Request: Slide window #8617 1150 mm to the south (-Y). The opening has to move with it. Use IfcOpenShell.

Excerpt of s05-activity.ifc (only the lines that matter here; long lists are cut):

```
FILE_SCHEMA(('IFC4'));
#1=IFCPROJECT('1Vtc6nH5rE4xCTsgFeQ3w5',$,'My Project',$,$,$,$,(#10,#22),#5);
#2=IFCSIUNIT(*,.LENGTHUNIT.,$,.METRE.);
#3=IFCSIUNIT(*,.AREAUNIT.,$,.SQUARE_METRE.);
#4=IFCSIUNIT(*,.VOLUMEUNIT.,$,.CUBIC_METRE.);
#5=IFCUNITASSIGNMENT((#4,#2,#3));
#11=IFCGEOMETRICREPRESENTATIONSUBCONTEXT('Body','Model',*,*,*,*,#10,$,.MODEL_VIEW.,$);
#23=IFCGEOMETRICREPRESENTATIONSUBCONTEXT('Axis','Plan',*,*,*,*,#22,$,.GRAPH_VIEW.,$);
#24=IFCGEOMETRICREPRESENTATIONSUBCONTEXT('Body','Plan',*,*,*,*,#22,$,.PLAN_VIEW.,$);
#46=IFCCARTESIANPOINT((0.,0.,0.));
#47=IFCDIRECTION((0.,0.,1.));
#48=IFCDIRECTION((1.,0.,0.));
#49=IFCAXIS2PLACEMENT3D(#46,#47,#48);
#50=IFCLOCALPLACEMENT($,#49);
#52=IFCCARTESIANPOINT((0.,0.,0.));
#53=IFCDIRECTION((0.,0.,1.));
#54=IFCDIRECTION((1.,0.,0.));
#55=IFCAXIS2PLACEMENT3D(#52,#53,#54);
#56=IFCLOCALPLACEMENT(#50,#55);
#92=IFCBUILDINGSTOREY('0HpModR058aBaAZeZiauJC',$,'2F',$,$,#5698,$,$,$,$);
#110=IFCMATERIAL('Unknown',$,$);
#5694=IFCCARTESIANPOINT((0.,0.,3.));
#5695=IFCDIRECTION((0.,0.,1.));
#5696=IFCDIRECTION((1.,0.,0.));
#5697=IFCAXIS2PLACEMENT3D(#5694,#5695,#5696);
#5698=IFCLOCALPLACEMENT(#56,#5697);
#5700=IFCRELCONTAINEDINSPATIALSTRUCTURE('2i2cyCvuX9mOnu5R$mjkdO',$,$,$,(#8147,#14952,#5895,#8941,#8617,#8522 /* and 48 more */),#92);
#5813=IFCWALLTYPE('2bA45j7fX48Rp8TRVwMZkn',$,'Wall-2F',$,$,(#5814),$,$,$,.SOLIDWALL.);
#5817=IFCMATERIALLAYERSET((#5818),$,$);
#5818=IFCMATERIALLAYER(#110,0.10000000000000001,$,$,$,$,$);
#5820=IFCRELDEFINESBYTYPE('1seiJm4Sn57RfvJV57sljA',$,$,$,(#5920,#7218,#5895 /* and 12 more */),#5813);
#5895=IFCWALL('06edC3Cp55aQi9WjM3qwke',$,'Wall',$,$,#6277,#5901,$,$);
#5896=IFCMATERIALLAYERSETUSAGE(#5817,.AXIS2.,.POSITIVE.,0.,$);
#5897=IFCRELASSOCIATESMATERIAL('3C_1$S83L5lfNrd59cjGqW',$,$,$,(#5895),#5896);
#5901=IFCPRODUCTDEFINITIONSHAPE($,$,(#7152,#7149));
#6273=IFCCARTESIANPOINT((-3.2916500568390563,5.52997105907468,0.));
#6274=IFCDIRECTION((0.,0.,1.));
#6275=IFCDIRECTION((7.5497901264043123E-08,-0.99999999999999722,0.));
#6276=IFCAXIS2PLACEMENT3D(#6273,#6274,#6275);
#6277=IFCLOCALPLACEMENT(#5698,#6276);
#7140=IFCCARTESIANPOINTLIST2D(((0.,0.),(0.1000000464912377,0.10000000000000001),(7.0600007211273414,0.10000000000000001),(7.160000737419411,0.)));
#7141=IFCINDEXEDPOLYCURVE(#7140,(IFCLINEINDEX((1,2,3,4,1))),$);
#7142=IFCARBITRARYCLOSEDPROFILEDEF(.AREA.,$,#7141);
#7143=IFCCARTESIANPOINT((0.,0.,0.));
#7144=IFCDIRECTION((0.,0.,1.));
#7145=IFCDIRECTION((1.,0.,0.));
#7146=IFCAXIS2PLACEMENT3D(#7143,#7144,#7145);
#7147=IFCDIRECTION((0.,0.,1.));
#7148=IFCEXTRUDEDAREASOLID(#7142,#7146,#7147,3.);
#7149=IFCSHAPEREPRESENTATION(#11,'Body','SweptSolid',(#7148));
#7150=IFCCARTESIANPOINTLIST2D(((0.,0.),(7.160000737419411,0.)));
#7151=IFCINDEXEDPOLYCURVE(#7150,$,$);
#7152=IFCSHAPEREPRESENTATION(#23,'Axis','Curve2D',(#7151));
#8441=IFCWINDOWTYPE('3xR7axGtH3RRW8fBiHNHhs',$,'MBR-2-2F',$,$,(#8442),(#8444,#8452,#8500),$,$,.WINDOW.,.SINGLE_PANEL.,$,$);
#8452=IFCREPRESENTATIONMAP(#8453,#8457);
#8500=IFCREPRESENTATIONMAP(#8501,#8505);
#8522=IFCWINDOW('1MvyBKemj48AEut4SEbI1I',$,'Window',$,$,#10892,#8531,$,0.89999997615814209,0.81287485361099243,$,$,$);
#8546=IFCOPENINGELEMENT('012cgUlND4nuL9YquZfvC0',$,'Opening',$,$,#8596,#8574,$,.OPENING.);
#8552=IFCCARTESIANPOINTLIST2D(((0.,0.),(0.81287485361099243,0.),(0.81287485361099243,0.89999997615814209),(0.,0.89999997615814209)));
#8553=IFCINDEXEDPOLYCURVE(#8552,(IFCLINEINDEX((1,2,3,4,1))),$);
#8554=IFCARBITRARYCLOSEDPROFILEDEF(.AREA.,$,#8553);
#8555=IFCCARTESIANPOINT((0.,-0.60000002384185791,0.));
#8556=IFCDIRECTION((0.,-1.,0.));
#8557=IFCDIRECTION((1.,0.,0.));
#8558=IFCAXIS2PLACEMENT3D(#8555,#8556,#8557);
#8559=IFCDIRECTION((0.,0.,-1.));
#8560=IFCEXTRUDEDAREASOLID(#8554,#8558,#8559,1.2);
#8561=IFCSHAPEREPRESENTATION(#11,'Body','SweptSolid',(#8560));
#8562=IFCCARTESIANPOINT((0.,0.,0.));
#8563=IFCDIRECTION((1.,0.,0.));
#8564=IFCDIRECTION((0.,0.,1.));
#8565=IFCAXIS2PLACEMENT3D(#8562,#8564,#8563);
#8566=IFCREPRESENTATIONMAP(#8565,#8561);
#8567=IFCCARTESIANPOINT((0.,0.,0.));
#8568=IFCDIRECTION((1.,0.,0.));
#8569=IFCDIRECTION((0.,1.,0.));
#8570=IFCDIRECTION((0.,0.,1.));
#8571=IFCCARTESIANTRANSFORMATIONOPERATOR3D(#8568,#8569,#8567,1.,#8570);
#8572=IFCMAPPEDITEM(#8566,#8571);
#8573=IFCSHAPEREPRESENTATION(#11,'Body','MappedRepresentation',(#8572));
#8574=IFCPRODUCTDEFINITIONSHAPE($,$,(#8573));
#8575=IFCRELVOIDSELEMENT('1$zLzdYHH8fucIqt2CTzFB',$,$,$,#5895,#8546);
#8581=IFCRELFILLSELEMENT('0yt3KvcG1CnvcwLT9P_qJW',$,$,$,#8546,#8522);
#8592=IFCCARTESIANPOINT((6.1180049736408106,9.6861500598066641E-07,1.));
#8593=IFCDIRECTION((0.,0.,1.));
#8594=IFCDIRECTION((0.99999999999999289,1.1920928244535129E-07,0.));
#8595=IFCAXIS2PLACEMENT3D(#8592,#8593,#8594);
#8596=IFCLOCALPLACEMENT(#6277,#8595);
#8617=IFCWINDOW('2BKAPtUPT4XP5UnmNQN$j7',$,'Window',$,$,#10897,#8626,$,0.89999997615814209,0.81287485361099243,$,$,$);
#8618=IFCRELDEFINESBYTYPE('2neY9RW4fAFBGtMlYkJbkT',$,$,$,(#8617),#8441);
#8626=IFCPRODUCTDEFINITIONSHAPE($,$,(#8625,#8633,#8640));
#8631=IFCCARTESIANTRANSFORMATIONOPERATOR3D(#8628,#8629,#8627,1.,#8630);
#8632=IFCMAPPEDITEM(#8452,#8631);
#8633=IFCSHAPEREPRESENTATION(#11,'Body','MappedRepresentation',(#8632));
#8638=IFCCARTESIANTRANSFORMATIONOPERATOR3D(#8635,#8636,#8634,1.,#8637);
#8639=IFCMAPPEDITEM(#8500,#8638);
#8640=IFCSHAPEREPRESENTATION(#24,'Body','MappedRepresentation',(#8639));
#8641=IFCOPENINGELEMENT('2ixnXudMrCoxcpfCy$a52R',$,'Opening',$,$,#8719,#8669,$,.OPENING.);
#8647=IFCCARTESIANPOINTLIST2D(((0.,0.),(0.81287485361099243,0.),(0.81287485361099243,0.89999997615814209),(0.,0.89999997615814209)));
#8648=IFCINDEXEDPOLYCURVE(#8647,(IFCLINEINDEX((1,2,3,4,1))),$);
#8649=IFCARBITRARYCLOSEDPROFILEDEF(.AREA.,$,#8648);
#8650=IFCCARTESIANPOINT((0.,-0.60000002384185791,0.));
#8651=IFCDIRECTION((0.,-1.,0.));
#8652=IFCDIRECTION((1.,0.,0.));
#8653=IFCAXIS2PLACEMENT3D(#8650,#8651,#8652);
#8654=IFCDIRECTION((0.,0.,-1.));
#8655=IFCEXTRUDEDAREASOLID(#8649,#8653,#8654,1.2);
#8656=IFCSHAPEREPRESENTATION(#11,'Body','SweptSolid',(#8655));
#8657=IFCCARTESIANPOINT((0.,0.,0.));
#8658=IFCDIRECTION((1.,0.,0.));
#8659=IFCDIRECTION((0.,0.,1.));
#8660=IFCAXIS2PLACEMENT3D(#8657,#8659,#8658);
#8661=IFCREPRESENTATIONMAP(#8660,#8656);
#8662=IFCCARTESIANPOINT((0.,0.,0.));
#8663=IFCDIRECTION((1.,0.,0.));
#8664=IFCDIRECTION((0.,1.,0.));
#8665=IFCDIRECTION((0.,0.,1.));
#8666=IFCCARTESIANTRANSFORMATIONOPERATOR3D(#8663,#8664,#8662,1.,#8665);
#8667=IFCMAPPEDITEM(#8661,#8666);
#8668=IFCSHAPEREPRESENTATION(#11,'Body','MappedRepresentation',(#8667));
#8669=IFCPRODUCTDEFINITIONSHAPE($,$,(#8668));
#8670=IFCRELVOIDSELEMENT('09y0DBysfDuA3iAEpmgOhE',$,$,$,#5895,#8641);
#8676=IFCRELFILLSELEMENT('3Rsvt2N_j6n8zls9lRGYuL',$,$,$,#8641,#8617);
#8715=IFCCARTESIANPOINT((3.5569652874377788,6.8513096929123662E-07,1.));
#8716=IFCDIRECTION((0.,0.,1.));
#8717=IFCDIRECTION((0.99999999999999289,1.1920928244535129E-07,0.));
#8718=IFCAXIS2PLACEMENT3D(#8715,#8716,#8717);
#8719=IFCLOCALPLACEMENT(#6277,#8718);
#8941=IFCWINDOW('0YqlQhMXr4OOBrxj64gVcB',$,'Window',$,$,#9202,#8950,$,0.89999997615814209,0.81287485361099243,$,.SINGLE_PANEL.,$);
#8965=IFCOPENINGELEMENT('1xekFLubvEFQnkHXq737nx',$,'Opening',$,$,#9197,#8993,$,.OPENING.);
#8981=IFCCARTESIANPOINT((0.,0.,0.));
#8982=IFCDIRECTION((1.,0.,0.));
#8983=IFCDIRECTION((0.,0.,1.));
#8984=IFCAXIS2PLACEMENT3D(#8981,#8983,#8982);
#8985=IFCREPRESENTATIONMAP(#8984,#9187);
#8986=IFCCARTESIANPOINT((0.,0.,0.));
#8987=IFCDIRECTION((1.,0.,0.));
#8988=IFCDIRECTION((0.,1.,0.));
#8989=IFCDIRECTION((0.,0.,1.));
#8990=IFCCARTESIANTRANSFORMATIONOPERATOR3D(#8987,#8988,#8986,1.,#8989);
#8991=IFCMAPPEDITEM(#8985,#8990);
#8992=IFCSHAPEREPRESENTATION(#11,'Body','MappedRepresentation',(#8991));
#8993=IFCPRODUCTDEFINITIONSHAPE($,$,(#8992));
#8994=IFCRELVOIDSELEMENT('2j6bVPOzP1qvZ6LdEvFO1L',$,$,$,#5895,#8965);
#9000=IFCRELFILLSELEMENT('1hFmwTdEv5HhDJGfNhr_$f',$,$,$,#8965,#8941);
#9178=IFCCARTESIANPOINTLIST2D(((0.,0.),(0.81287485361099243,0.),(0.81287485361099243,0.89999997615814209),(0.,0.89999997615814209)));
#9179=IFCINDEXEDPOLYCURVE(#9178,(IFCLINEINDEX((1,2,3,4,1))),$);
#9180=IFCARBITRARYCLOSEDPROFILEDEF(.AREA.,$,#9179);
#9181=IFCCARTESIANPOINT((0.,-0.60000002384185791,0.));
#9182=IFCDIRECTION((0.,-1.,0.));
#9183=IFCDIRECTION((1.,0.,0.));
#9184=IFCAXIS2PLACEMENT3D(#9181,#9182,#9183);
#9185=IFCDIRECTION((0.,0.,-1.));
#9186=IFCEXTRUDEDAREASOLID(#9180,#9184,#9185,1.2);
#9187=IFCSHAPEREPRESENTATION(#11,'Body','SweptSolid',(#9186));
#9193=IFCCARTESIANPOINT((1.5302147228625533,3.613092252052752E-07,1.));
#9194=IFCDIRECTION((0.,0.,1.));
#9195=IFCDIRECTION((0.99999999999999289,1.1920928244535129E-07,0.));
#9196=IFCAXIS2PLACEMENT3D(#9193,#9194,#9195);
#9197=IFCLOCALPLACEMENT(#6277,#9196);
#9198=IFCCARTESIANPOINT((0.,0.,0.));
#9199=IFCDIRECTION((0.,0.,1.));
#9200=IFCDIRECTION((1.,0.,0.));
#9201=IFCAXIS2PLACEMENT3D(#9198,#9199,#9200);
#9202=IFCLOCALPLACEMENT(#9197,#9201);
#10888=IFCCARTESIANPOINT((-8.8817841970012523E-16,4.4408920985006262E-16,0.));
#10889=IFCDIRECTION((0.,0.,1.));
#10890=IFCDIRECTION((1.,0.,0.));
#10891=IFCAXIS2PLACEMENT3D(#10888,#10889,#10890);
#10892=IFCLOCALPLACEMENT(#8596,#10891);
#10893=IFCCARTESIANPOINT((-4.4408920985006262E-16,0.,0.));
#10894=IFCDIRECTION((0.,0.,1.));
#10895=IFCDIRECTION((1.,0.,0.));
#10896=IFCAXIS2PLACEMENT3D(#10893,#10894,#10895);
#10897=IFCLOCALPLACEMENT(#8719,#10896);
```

```python
import ifcopenshell
import ifcopenshell.api.geometry
import ifcopenshell.util.placement
import ifcopenshell.util.unit

model = ifcopenshell.open("s05-activity.ifc")
unit_scale = ifcopenshell.util.unit.calculate_unit_scale(model)

window = model.by_guid("2BKAPtUPT4XP5UnmNQN$j7")
opening = window.FillsVoids[0].RelatingOpeningElement
wall = opening.VoidsElements[0].RelatingBuildingElement

wall_matrix = ifcopenshell.util.placement.get_local_placement(wall.ObjectPlacement)
shift = wall_matrix[:3, 0] * 1.15 / unit_scale
before = ifcopenshell.util.placement.get_local_placement(window.ObjectPlacement)[:3, 3].copy()

# The window is placed relative to its opening, so it follows when the opening moves.
matrix = ifcopenshell.util.placement.get_local_placement(opening.ObjectPlacement)
matrix[:3, 3] += shift
ifcopenshell.api.geometry.edit_object_placement(
    model, product=opening, matrix=matrix, is_si=False, should_transform_children=True
)

after = ifcopenshell.util.placement.get_local_placement(window.ObjectPlacement)[:3, 3]
print("window moved by", (after - before).round(3) + 0.0)

model.write("s05-activity_rev.ifc")
```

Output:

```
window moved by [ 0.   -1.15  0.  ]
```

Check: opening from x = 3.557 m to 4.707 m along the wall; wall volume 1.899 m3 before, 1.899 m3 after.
